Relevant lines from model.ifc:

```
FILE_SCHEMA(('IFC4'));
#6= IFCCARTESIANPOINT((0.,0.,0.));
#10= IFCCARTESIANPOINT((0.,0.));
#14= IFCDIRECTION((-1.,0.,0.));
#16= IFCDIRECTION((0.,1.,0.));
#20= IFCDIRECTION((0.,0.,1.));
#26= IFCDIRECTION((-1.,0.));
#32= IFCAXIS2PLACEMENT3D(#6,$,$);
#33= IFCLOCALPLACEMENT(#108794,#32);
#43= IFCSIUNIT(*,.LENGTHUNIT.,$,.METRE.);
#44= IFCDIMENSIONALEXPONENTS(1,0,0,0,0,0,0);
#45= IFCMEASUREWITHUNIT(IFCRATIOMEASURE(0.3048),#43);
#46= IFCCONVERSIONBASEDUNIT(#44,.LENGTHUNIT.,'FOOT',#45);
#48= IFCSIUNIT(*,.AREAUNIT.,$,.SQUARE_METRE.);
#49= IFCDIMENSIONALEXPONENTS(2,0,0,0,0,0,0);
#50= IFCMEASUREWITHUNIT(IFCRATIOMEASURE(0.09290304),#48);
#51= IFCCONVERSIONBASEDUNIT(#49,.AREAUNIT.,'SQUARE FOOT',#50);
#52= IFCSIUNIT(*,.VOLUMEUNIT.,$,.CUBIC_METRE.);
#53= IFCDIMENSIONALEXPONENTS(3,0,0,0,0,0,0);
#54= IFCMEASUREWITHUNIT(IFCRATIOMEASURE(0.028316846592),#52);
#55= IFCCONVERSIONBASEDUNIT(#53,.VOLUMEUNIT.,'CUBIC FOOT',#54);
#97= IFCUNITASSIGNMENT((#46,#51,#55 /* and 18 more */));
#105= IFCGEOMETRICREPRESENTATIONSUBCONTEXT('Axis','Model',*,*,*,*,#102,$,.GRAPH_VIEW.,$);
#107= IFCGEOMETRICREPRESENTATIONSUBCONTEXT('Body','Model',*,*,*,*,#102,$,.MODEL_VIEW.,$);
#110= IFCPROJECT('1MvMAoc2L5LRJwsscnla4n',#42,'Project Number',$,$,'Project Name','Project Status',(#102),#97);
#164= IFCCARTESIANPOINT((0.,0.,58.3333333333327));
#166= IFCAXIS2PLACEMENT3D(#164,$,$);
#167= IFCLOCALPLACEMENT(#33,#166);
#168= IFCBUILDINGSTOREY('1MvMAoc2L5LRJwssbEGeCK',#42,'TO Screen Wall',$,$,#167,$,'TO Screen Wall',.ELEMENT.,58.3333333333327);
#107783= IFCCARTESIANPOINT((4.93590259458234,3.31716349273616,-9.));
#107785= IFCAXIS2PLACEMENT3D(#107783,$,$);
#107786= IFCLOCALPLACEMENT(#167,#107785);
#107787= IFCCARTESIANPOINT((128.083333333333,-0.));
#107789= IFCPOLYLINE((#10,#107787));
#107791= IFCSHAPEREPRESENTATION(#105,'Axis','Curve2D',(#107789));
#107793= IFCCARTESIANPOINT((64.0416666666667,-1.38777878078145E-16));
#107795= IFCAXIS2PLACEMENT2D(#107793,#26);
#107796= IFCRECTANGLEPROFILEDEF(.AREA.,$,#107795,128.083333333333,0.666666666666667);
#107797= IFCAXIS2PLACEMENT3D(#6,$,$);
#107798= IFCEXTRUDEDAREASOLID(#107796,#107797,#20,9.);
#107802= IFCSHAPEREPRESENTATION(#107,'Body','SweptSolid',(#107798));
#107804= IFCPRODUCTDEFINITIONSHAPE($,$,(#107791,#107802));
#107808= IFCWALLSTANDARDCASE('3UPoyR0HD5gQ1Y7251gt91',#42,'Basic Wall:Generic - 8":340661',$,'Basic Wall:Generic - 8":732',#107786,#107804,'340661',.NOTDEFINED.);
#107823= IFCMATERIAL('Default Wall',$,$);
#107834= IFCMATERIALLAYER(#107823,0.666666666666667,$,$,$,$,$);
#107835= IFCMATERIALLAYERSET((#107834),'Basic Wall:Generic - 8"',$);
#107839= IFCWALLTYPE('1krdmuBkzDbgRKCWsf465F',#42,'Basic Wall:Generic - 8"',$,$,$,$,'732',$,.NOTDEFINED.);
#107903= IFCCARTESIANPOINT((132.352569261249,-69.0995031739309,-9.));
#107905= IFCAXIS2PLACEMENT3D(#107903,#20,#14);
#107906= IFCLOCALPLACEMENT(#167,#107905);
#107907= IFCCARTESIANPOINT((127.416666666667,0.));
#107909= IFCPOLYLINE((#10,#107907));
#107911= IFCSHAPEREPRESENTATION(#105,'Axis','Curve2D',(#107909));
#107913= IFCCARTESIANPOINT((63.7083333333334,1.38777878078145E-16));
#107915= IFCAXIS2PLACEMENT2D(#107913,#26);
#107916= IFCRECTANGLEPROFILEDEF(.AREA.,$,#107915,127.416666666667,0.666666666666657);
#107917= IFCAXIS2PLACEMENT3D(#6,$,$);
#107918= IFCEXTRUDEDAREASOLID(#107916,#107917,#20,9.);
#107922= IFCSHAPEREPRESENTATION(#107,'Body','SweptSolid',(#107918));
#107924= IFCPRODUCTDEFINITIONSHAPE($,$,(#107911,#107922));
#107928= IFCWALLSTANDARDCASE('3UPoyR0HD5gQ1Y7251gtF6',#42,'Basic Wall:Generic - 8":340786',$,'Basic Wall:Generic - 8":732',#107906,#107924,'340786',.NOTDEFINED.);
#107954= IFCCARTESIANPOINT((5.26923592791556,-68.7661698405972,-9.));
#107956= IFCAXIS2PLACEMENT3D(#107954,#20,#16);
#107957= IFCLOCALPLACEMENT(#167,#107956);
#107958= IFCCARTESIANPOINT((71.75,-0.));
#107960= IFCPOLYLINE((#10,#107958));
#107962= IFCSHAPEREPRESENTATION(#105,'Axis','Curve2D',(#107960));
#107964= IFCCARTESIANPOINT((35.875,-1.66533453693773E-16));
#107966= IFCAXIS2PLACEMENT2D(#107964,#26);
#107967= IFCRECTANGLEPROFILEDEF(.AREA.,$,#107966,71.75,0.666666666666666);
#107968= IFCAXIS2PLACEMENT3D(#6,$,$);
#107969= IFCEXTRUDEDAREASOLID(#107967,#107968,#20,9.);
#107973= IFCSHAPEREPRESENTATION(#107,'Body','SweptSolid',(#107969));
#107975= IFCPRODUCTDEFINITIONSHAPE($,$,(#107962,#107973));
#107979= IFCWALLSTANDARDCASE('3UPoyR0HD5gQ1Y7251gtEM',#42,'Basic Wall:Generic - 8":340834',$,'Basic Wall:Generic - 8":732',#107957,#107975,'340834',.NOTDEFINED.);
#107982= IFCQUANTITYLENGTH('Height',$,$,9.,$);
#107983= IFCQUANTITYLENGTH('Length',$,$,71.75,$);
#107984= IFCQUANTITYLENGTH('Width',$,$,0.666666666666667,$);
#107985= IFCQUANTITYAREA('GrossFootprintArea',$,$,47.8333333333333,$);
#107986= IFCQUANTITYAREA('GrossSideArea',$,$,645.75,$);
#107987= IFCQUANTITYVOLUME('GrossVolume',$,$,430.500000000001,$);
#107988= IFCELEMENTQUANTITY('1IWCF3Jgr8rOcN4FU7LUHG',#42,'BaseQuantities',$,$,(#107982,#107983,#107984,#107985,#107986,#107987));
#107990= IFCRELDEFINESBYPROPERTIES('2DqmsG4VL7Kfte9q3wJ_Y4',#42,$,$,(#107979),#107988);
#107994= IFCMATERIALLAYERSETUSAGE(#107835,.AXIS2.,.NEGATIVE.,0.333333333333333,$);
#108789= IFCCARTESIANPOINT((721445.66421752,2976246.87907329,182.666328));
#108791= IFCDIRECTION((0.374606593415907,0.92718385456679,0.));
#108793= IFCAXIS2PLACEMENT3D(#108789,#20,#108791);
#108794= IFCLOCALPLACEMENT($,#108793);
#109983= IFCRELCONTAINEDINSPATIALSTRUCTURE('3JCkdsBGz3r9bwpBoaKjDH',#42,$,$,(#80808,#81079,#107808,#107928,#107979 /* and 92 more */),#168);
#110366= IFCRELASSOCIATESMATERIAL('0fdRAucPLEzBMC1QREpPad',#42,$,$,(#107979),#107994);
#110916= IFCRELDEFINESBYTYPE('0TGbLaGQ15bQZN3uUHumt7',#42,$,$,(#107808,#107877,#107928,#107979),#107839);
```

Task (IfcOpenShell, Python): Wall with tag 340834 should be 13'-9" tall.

```python
import ifcopenshell
import ifcopenshell.api.pset
import ifcopenshell.geom
import ifcopenshell.util.element
import ifcopenshell.util.representation
import ifcopenshell.util.shape
import ifcopenshell.util.unit

model = ifcopenshell.open("model.ifc")
unit_scale = ifcopenshell.util.unit.calculate_unit_scale(model)
area_scale = ifcopenshell.util.unit.calculate_unit_scale(model, "AREAUNIT")
volume_scale = ifcopenshell.util.unit.calculate_unit_scale(model, "VOLUMEUNIT")
settings = ifcopenshell.geom.settings()


def volume(element):
    """Net volume in cubic metres, openings subtracted."""
    shape = ifcopenshell.geom.create_shape(settings, element)
    return ifcopenshell.util.shape.get_volume(shape.geometry)


wall = model.by_guid("3UPoyR0HD5gQ1Y7251gtEM")
before = volume(wall)

body = ifcopenshell.util.representation.get_representation(wall, "Model", "Body")
solid = body.Items[0]
old_height = solid.Depth
solid.Depth = 165 * 0.0254 / unit_scale
after = volume(wall)

# Update the stored height, areas and volumes.
qto = model.by_id(ifcopenshell.util.element.get_pset(wall, "BaseQuantities", should_inherit=False)["id"])
ifcopenshell.api.pset.edit_qto(model, qto=qto, properties={
    "Height": solid.Depth,
    "GrossSideArea": ifcopenshell.util.element.get_pset(wall, "BaseQuantities", "GrossSideArea") * solid.Depth / old_height,
    "GrossVolume": ifcopenshell.util.element.get_pset(wall, "BaseQuantities", "GrossVolume") * solid.Depth / old_height,
})

print(f"height {old_height:g} -> {solid.Depth:g}, volume {before:.3f} -> {after:.3f} m3")

model.write("model_rev.ifc")
```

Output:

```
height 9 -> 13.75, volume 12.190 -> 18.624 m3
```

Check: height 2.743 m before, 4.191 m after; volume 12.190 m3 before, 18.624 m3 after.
